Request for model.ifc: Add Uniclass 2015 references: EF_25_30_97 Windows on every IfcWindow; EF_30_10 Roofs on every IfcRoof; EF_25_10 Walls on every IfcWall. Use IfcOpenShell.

First a look at what the model holds.

```python
import ifcopenshell

model = ifcopenshell.open("model.ifc")
print(model.schema)
print("classifications:", [c.Name for c in model.by_type("IfcClassification")])
for ifc_class in ("IfcDoor", "IfcRoof", "IfcStair", "IfcWall", "IfcWindow"):
    print(ifc_class, len(model.by_type(ifc_class)))
```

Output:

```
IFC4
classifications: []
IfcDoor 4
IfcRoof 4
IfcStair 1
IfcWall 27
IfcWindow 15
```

```python
import ifcopenshell
import ifcopenshell.api.classification

model = ifcopenshell.open("model.ifc")

system = ifcopenshell.api.classification.add_classification(model, classification="Uniclass 2015")

codes = {
    "IfcWindow": ("EF_25_30_97", "Windows"),
    "IfcRoof": ("EF_30_10", "Roofs"),
    "IfcWall": ("EF_25_10", "Walls"),
}
for ifc_class, (code, name) in codes.items():
    products = model.by_type(ifc_class)
    ifcopenshell.api.classification.add_reference(
        model, products=products, classification=system, identification=code, name=name
    )
    print(code, len(products))

model.write("model_v2.ifc")
```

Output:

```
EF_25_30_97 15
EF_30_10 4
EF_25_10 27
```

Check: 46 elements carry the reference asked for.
